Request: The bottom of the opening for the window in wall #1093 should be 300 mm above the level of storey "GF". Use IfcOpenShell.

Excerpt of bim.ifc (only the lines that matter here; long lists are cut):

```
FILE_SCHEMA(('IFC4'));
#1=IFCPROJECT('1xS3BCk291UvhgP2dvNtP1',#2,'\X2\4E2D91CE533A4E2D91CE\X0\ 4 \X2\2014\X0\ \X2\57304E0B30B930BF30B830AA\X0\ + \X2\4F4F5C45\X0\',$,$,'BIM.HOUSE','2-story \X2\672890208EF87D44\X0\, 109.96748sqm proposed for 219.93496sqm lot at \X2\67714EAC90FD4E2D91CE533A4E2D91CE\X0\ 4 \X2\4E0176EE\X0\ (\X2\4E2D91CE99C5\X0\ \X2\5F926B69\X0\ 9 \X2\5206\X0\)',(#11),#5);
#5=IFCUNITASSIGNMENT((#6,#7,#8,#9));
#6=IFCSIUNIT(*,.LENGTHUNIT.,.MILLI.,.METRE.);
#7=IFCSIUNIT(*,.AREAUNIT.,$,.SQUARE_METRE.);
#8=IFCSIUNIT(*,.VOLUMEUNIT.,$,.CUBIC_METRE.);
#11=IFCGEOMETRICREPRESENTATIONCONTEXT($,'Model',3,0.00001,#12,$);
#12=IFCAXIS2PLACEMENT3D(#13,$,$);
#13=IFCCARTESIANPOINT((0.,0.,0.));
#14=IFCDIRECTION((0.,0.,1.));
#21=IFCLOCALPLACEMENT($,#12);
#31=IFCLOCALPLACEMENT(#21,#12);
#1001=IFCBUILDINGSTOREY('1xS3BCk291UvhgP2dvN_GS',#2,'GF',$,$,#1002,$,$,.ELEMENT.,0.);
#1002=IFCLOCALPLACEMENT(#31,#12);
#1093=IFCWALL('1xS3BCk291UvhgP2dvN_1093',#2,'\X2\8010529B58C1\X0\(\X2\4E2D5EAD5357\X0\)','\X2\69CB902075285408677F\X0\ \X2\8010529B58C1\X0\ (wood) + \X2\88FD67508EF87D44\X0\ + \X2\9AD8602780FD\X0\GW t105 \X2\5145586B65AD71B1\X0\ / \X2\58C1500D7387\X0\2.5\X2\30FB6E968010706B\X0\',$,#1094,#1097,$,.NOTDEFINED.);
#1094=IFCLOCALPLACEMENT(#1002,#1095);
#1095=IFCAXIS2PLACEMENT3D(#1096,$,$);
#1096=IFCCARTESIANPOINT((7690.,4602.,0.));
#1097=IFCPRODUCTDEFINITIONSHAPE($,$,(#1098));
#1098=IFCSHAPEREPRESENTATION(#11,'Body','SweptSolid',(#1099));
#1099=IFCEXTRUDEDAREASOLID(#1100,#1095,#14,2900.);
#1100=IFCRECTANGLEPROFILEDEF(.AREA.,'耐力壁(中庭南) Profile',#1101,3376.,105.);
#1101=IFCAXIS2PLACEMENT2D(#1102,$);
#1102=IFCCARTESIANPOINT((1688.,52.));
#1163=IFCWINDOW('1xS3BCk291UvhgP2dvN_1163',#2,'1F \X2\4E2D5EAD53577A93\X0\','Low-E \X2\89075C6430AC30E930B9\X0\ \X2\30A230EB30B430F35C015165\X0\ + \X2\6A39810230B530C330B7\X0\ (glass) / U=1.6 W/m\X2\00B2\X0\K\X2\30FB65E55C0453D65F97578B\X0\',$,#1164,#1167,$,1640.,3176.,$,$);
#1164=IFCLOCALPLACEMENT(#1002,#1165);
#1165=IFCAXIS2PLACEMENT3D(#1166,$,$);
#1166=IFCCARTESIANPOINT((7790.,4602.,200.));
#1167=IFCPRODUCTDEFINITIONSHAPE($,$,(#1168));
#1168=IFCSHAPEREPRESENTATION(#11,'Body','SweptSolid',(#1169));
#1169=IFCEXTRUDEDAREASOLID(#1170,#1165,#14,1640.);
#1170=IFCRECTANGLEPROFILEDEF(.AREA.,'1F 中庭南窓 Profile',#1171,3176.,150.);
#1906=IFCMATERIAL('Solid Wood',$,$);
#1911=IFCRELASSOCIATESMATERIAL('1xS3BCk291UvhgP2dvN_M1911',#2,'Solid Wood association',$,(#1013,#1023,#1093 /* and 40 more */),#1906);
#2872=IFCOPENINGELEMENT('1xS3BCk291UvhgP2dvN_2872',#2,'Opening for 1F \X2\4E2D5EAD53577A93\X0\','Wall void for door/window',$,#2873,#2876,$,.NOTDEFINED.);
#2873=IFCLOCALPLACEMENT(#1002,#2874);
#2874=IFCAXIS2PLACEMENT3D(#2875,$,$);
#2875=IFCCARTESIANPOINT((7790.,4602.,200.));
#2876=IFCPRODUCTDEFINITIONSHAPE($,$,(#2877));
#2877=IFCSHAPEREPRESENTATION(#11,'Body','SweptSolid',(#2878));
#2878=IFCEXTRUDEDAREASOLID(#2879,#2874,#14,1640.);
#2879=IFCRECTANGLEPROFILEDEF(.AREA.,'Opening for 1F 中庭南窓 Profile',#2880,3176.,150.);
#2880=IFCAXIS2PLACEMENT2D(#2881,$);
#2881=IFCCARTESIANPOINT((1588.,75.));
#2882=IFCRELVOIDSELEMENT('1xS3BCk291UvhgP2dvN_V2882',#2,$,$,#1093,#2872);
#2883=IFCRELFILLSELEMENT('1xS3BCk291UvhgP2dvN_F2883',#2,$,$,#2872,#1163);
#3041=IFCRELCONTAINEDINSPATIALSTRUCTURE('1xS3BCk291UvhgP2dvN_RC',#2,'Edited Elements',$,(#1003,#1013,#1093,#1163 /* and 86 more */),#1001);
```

```python
import numpy as np
import ifcopenshell
import ifcopenshell.api.geometry
import ifcopenshell.geom
import ifcopenshell.util.element
import ifcopenshell.util.placement
import ifcopenshell.util.shape
import ifcopenshell.util.unit

model = ifcopenshell.open("bim.ifc")
unit_scale = ifcopenshell.util.unit.calculate_unit_scale(model)

window = model.by_id(1163)
opening = window.FillsVoids[0].RelatingOpeningElement
storey = ifcopenshell.util.element.get_container(window, ifc_class="IfcBuildingStorey")
level = ifcopenshell.util.placement.get_local_placement(storey.ObjectPlacement)[2, 3]

# The opening's origin need not be at the sill, so measure its lowest point.
shape = ifcopenshell.geom.create_shape(ifcopenshell.geom.settings(), opening)
bottom = ifcopenshell.util.shape.get_shape_bottom_elevation(shape, shape.geometry) / unit_scale
dz = level + 300.0 - bottom

shift = np.array([0.0, 0.0, dz])
# The window is not placed relative to its opening, so move both.
for product in (opening, window):
    matrix = ifcopenshell.util.placement.get_local_placement(product.ObjectPlacement)
    matrix[:3, 3] += shift
    ifcopenshell.api.geometry.edit_object_placement(model, product=product, matrix=matrix, is_si=False)

print(f"moved by {dz * unit_scale:+.3f} m")

model.write("bim_edited.ifc")
```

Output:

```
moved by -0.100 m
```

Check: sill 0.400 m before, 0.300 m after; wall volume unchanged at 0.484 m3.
